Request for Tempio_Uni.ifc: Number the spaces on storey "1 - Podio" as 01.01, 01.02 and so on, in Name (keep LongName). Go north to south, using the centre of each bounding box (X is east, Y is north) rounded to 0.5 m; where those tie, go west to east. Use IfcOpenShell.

First a look at what the model holds.

```python
import ifcopenshell
import ifcopenshell.util.element
import ifcopenshell.util.placement

model = ifcopenshell.open("Tempio_Uni.ifc")
print(model.schema)
storey = next(s for s in model.by_type("IfcBuildingStorey") if s.Name == "1 - Podio")
spaces = [e for e in ifcopenshell.util.element.get_decomposition(storey) if e.is_a("IfcSpace")]
for e in sorted(spaces, key=lambda e: e.id()):
    origin = ifcopenshell.util.placement.get_local_placement(e.ObjectPlacement)[:3, 3]
    print(e.id(), e.Name, e.LongName, origin.round(2) + 0.0, sep=" | ")
```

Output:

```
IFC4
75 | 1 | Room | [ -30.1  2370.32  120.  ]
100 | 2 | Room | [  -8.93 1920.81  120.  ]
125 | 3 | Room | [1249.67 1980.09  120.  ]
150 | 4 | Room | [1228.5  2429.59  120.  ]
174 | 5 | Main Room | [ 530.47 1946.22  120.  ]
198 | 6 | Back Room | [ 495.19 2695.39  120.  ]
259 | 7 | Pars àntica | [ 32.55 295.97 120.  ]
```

```python
import ifcopenshell
import ifcopenshell.geom
import ifcopenshell.util.element
import ifcopenshell.util.shape

model = ifcopenshell.open("Tempio_Uni.ifc")
settings = ifcopenshell.geom.settings()
settings.set("use-world-coords", True)


def centre(element):
    shape = ifcopenshell.geom.create_shape(settings, element)
    return ifcopenshell.util.shape.get_bbox_centroid(shape.geometry)


storey = next(s for s in model.by_type("IfcBuildingStorey") if s.Name == "1 - Podio")
spaces = [e for e in ifcopenshell.util.element.get_decomposition(storey) if e.is_a("IfcSpace")]

# Insertion points can sit at a corner or the storey origin, so sort by the geometry (in metres).
centres = {e: centre(e) for e in spaces}
spaces.sort(key=lambda e: (-round(centres[e][1] / 0.5), centres[e][0]))

for i, e in enumerate(spaces, start=1):
    number = f"01.{i:02d}"
    e.Name = number
    print(e.id(), number)

model.write("Tempio_Uni_updated.ifc")
```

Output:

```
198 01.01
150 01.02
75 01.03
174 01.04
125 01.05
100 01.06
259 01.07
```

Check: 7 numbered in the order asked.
